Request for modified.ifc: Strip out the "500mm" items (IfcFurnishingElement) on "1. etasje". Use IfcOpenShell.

First a look at what the model holds.

```python
import ifcopenshell
import ifcopenshell.util.element

model = ifcopenshell.open("modified.ifc")
print(model.schema)
storey = next(s for s in model.by_type("IfcBuildingStorey") if s.Name == "1. etasje")
furniture = [e for e in ifcopenshell.util.element.get_decomposition(storey) if e.is_a("IfcFurnishingElement")]
seen = {}
for e in furniture:
    element_type = ifcopenshell.util.element.get_type(e)
    name = element_type.Name if element_type not in (None, e) else None
    seen[name] = seen.get(name, 0) + 1
for name, count in sorted(seen.items(), key=str):
    print(count, "x", name)
```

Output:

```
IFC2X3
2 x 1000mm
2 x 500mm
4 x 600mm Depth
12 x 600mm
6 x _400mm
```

```python
import ifcopenshell
import ifcopenshell.api.root
import ifcopenshell.util.element

model = ifcopenshell.open("modified.ifc")

storey = next(s for s in model.by_type("IfcBuildingStorey") if s.Name == "1. etasje")
furniture = [e for e in ifcopenshell.util.element.get_decomposition(storey) if e.is_a("IfcFurnishingElement")]
targets = [e for e in furniture if (t := ifcopenshell.util.element.get_type(e)) not in (None, e) and t.Name == "500mm"]

for e in targets:
    ifcopenshell.api.root.remove_product(model, product=e)
print(len(targets), "removed")

model.write("modified_edited.ifc")
```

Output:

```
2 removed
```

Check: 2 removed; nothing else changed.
